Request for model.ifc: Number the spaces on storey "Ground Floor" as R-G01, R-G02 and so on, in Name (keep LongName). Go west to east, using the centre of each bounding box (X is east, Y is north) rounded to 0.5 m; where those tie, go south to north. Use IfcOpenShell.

First a look at what the model holds.

```python
import ifcopenshell
import ifcopenshell.util.element
import ifcopenshell.util.placement

model = ifcopenshell.open("model.ifc")
print(model.schema)
storey = next(s for s in model.by_type("IfcBuildingStorey") if s.Name == "Ground Floor")
spaces = [e for e in ifcopenshell.util.element.get_decomposition(storey) if e.is_a("IfcSpace")]
for e in sorted(spaces, key=lambda e: e.id()):
    origin = ifcopenshell.util.placement.get_local_placement(e.ObjectPlacement)[:3, 3]
    print(e.id(), e.Name, e.LongName, origin.round(2) + 0.0, sep=" | ")
```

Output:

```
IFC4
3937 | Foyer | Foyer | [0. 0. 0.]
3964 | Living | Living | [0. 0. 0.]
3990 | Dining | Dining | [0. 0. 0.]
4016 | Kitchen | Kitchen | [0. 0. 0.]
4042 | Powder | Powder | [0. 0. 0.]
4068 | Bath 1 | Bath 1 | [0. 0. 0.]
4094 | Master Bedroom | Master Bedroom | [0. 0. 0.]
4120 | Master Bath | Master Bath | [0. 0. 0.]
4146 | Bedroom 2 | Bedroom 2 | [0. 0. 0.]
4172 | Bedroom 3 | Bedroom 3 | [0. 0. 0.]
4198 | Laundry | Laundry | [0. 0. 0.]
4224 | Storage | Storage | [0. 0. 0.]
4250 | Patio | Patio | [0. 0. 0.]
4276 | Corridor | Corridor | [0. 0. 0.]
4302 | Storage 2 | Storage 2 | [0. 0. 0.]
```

```python
import ifcopenshell
import ifcopenshell.geom
import ifcopenshell.util.element
import ifcopenshell.util.shape

model = ifcopenshell.open("model.ifc")
settings = ifcopenshell.geom.settings()
settings.set("use-world-coords", True)


def centre(element):
    shape = ifcopenshell.geom.create_shape(settings, element)
    return ifcopenshell.util.shape.get_bbox_centroid(shape.geometry)


storey = next(s for s in model.by_type("IfcBuildingStorey") if s.Name == "Ground Floor")
spaces = [e for e in ifcopenshell.util.element.get_decomposition(storey) if e.is_a("IfcSpace")]

# Insertion points can sit at a corner or the storey origin, so sort by the geometry (in metres).
centres = {e: centre(e) for e in spaces}
spaces.sort(key=lambda e: (round(centres[e][0] / 0.5), centres[e][1]))

for i, e in enumerate(spaces, start=1):
    number = f"R-G{i:02d}"
    e.Name = number
    print(e.id(), number)

model.write("model-out.ifc")
```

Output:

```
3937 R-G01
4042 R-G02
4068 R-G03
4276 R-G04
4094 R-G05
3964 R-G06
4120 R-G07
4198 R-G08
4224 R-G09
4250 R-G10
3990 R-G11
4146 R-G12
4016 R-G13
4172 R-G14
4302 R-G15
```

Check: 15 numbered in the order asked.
